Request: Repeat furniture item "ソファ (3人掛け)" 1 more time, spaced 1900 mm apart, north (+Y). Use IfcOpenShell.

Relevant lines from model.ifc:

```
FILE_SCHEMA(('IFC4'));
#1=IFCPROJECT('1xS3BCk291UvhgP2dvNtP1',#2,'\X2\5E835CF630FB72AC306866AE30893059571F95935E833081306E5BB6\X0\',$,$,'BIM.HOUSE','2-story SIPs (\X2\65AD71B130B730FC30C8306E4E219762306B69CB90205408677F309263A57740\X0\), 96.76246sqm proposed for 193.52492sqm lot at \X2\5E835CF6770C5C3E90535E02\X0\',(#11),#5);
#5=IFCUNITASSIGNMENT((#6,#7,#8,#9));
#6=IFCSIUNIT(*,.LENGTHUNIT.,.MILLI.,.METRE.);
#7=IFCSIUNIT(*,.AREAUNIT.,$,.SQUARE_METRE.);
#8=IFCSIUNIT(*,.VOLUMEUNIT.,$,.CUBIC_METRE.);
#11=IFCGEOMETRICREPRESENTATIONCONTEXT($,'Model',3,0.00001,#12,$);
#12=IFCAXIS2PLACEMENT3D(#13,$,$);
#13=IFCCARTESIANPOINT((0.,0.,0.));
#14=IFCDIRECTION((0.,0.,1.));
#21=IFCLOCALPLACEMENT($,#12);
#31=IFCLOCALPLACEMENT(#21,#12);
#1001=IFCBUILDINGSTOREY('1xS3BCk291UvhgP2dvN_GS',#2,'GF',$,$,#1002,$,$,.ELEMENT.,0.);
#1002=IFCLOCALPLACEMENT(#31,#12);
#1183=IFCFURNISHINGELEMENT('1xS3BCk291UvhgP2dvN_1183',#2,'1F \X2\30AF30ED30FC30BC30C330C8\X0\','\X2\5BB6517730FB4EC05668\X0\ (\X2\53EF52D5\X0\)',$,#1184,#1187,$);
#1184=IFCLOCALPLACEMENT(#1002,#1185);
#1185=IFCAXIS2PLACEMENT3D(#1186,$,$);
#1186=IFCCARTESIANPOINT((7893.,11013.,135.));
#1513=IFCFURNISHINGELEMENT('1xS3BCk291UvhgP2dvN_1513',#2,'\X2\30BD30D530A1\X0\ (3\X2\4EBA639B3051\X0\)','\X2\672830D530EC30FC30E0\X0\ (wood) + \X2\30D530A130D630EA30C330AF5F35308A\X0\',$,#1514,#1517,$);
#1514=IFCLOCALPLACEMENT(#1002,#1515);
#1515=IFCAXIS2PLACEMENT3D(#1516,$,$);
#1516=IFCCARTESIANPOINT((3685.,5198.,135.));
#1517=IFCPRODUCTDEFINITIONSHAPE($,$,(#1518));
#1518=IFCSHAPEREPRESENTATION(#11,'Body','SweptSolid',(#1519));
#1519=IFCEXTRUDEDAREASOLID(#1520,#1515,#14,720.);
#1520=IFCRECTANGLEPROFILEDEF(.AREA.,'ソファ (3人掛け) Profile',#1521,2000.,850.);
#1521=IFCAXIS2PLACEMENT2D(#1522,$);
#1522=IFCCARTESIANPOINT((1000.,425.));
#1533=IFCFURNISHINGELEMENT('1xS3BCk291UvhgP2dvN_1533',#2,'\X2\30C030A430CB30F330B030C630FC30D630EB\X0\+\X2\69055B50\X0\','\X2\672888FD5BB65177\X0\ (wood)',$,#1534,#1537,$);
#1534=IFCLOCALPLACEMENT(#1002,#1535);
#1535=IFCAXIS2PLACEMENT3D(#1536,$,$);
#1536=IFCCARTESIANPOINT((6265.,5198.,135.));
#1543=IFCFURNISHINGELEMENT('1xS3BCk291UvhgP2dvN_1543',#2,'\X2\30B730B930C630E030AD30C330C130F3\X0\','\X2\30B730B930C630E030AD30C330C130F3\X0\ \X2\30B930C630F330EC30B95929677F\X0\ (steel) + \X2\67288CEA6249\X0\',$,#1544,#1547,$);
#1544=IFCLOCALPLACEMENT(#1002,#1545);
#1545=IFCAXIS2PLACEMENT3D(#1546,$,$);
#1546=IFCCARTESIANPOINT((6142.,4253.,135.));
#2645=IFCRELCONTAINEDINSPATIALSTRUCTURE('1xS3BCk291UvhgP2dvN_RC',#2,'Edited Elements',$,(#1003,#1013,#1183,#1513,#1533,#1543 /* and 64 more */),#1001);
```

```python
import numpy as np
import ifcopenshell
import ifcopenshell.api.geometry
import ifcopenshell.api.root
import ifcopenshell.util.element
import ifcopenshell.util.placement
import ifcopenshell.util.unit

model = ifcopenshell.open("model.ifc")
unit_scale = ifcopenshell.util.unit.calculate_unit_scale(model)


def reuse_history(source, copy):
    """copy_class also copies each property set's owner history, people and application; keep the originals."""
    for rel in copy.IsDefinedBy:
        if rel.is_a("IfcRelDefinesByProperties") and (history := rel.RelatingPropertyDefinition.OwnerHistory):
            rel.RelatingPropertyDefinition.OwnerHistory = source.OwnerHistory
            ifcopenshell.util.element.remove_deep2(model, history)


source = model.by_guid("1xS3BCk291UvhgP2dvN_1513")
base = ifcopenshell.util.placement.get_local_placement(source.ObjectPlacement)
step = np.array([0.0, 1.0, 0.0]) * 1.9 / unit_scale

for i in range(1, 2):
    copy = ifcopenshell.api.root.copy_class(model, product=source)
    copy.Representation = ifcopenshell.util.element.copy_deep(
        model, source.Representation, exclude=["IfcGeometricRepresentationContext", "IfcRepresentationMap"]
    )
    reuse_history(source, copy)
    matrix = base.copy()
    matrix[:3, 3] += i * step
    print("added at", matrix[:3, 3].round(3) + 0.0)
    ifcopenshell.api.geometry.edit_object_placement(model, product=copy, matrix=matrix, is_si=False)

model.write("model_edited.ifc")
```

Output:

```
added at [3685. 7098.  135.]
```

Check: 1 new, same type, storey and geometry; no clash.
